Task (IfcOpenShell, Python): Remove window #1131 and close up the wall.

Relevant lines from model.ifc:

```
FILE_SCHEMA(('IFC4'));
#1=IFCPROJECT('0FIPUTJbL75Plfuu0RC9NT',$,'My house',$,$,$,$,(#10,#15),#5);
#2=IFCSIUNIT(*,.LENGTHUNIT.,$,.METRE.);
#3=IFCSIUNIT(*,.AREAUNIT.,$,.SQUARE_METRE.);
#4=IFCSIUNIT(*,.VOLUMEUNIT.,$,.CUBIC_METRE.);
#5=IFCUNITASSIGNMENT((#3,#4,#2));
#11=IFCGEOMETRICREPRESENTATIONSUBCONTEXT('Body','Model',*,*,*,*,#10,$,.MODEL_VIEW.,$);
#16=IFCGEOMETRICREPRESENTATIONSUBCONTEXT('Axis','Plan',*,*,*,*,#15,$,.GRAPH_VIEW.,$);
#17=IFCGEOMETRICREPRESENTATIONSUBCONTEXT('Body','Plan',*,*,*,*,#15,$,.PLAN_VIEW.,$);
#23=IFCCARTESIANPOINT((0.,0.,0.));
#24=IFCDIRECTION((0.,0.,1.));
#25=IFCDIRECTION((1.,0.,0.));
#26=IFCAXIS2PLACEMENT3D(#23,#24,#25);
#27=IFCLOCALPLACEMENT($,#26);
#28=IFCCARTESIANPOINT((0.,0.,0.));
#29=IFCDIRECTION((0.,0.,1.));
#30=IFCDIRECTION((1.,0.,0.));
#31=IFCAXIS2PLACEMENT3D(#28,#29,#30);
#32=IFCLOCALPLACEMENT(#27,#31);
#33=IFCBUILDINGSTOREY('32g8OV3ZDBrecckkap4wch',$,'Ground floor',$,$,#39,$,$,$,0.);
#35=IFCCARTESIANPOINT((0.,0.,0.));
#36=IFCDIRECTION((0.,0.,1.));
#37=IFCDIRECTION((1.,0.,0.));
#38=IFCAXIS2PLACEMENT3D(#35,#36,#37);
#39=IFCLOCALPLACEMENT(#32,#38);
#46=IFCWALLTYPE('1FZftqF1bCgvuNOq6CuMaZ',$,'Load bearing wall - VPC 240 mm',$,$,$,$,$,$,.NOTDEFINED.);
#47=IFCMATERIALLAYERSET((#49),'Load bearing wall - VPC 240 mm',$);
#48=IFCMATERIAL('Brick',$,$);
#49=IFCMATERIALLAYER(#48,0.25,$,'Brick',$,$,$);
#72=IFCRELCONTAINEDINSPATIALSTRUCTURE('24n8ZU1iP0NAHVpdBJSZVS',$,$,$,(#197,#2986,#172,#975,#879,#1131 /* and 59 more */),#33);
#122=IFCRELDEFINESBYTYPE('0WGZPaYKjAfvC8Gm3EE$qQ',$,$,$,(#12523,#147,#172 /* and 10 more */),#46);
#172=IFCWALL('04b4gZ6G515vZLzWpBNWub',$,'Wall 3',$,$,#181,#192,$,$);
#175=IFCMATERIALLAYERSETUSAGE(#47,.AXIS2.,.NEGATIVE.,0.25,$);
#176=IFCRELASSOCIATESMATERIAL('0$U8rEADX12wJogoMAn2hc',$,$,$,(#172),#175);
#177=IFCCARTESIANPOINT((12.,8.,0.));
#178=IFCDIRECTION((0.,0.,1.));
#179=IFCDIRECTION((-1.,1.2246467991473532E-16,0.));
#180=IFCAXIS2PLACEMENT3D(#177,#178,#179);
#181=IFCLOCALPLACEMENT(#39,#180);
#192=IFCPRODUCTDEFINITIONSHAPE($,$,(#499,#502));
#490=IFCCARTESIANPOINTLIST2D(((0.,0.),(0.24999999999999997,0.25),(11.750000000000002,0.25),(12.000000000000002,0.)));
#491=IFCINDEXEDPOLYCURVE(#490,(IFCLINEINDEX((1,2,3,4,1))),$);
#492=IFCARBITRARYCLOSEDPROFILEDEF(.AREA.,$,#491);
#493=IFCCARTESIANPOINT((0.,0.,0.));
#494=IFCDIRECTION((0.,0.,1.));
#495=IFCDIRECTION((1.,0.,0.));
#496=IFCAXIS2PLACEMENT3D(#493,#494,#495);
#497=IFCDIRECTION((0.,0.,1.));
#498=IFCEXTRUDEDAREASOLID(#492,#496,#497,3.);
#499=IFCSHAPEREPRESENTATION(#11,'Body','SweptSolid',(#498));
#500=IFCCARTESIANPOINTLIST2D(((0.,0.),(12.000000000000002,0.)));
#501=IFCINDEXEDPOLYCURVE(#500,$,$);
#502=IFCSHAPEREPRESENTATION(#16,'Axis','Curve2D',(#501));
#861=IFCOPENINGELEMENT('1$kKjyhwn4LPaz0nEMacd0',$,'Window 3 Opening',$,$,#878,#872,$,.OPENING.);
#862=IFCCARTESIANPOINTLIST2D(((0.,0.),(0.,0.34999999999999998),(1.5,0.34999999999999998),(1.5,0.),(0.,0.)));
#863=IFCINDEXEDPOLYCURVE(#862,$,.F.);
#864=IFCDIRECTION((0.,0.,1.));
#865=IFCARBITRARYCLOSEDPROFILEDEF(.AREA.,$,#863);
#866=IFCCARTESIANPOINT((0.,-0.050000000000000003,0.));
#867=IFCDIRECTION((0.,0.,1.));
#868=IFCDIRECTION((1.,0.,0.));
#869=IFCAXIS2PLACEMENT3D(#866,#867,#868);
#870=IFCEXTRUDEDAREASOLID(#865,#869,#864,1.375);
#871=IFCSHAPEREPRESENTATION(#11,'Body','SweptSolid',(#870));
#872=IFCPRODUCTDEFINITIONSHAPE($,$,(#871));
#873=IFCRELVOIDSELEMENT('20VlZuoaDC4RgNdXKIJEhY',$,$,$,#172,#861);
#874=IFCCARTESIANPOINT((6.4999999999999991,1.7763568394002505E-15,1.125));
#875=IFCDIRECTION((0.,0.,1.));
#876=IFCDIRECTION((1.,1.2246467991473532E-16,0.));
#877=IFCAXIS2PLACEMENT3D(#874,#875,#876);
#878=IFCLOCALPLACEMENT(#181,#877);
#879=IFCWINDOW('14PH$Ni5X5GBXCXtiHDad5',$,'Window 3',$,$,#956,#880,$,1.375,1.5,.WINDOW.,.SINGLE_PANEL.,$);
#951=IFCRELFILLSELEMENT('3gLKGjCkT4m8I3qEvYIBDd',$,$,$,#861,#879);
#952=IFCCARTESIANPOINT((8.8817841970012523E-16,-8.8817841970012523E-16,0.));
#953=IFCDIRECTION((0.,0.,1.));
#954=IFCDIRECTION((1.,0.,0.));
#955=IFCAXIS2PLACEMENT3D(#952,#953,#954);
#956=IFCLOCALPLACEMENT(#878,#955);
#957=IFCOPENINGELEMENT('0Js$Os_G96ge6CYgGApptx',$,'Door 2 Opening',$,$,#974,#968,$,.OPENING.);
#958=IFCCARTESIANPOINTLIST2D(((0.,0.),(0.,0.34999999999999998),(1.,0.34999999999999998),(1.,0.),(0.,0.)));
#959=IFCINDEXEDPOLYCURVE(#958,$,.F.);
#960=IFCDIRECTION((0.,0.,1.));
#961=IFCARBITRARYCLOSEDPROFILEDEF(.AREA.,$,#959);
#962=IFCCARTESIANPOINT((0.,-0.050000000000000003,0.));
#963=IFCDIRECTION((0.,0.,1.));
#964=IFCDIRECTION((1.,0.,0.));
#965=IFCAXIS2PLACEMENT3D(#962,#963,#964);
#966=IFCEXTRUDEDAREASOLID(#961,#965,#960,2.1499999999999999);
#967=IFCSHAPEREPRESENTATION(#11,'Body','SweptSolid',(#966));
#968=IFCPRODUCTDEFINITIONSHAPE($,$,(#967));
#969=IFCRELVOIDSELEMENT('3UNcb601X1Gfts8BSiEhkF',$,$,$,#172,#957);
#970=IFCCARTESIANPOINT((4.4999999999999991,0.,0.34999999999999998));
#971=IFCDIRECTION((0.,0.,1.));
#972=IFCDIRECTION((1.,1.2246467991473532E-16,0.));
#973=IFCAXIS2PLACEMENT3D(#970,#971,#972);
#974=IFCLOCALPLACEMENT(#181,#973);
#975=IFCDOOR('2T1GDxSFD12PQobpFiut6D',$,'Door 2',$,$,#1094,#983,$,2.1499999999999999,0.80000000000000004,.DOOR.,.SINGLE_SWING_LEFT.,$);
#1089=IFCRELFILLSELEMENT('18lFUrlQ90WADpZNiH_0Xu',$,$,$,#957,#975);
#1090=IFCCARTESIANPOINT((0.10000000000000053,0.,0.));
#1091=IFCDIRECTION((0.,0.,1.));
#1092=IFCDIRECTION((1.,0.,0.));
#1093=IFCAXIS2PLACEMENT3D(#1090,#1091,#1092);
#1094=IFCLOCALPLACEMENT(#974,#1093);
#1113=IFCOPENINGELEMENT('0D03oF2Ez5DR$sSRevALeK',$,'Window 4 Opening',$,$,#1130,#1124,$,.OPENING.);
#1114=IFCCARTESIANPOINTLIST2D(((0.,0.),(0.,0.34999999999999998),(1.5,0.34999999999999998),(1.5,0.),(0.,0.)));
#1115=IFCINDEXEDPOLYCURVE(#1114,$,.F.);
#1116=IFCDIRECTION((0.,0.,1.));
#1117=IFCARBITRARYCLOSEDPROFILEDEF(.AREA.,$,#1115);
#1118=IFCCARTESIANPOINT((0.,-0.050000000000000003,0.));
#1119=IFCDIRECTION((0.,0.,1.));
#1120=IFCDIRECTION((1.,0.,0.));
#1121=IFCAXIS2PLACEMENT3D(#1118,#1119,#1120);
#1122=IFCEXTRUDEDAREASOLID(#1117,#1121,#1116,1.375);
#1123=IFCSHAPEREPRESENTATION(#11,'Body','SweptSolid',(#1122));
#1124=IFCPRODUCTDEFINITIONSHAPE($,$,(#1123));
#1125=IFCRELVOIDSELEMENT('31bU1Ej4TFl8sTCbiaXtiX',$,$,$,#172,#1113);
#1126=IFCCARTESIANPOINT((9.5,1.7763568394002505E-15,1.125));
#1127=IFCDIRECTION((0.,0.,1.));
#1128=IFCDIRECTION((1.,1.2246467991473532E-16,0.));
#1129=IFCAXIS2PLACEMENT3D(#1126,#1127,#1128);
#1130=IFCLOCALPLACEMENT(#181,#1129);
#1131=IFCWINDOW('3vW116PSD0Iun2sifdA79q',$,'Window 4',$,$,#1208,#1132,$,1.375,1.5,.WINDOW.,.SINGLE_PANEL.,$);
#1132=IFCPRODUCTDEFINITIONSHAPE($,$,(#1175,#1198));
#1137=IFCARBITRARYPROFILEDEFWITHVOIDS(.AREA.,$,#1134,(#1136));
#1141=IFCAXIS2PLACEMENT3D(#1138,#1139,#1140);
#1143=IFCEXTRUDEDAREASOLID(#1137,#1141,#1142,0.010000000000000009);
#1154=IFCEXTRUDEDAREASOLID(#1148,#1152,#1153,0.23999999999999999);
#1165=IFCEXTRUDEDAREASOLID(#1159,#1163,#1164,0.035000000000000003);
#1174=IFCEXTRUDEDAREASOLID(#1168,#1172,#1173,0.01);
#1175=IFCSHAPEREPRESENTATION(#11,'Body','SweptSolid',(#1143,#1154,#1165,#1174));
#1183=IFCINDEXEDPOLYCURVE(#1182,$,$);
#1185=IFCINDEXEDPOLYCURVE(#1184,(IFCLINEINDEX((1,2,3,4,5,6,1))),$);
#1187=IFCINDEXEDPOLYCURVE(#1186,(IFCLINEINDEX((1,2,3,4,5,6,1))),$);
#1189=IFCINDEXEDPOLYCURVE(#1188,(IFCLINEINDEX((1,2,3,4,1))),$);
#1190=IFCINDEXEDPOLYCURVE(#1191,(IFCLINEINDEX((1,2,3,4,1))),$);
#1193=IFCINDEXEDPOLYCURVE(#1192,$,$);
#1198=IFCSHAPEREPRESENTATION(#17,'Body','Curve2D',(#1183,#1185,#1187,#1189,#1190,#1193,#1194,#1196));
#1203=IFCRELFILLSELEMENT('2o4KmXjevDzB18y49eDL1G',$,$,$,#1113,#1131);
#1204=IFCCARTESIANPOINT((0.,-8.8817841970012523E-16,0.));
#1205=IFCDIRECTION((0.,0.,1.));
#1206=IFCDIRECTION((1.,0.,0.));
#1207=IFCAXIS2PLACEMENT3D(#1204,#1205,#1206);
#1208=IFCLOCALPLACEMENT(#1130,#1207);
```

```python
import ifcopenshell
import ifcopenshell.api.feature
import ifcopenshell.api.root
import ifcopenshell.geom
import ifcopenshell.util.shape

model = ifcopenshell.open("model.ifc")
settings = ifcopenshell.geom.settings()


def volume(element):
    """Net volume in cubic metres, openings subtracted."""
    shape = ifcopenshell.geom.create_shape(settings, element)
    return ifcopenshell.util.shape.get_volume(shape.geometry)


window = model.by_guid("3vW116PSD0Iun2sifdA79q")
opening = window.FillsVoids[0].RelatingOpeningElement
wall = opening.VoidsElements[0].RelatingBuildingElement
before = volume(wall)

ifcopenshell.api.root.remove_product(model, product=window)
ifcopenshell.api.feature.remove_feature(model, feature=opening)

after = volume(wall)

print(f"wall volume {before:.3f} -> {after:.3f} m3")

model.write("model_v2.ifc")
```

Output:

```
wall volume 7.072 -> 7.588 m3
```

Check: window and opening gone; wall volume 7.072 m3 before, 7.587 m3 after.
